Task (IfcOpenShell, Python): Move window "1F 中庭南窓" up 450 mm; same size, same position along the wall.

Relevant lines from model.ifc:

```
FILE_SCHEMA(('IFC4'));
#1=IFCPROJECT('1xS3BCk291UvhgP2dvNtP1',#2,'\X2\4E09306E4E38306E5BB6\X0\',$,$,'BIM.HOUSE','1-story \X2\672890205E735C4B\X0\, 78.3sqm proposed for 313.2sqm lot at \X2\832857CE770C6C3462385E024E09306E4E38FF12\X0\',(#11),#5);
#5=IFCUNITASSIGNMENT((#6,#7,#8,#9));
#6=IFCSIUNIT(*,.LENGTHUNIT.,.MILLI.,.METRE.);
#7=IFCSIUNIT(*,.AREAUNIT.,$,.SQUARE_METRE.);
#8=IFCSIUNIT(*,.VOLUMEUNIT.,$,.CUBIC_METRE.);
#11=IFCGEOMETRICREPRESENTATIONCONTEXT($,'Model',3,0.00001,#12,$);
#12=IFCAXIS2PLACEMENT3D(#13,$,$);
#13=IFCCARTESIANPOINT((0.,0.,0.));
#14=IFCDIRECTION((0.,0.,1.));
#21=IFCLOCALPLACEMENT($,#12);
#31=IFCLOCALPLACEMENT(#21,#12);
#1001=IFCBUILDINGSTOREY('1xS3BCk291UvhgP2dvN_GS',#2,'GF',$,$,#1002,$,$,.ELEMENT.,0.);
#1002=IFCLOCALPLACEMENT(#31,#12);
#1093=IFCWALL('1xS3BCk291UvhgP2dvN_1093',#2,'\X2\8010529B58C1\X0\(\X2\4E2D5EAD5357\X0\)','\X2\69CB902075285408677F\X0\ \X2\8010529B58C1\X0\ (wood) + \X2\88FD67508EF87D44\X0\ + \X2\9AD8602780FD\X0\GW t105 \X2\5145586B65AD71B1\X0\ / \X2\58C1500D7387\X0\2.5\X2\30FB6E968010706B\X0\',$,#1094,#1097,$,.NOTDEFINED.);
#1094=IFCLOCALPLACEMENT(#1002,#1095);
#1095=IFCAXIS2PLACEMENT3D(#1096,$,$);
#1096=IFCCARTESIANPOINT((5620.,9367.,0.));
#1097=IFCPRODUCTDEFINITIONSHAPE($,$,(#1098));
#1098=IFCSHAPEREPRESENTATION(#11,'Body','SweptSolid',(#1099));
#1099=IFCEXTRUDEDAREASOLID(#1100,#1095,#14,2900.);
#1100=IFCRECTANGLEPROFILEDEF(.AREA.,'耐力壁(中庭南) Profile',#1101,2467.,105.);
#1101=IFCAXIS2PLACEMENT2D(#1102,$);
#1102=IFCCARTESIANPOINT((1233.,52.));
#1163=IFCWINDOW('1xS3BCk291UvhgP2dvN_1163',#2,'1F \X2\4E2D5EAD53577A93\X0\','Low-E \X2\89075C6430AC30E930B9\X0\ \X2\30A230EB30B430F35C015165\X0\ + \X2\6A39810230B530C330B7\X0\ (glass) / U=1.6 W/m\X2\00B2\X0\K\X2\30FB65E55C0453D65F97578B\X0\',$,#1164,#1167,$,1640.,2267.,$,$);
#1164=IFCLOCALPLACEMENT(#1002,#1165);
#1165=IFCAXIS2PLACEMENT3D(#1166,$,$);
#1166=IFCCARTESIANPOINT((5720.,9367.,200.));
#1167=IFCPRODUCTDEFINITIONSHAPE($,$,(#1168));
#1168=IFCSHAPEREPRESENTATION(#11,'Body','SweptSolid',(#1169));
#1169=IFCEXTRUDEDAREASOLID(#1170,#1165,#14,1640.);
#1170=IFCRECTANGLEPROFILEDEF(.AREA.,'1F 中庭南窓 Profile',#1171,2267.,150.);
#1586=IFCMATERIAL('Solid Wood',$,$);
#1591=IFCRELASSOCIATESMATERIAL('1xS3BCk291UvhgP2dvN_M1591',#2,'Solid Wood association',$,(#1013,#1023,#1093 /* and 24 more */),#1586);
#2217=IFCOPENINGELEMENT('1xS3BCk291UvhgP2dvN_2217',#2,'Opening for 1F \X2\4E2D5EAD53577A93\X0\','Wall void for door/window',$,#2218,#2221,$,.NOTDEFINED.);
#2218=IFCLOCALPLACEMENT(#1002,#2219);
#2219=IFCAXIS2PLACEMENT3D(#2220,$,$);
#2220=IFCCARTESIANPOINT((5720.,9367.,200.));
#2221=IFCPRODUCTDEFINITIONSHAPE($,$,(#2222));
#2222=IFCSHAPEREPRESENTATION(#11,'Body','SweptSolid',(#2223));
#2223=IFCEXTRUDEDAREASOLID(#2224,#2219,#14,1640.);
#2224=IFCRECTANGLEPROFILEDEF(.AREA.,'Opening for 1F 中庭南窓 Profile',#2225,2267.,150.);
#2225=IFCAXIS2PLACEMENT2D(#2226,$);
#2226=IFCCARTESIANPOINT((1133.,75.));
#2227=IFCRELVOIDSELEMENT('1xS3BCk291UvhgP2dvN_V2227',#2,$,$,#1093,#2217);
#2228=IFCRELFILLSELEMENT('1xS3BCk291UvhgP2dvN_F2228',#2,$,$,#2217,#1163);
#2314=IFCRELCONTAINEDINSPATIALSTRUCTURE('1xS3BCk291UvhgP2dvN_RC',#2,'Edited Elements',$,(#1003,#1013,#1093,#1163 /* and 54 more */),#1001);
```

```python
import numpy as np
import ifcopenshell
import ifcopenshell.api.geometry
import ifcopenshell.util.placement
import ifcopenshell.util.unit

model = ifcopenshell.open("model.ifc")
unit_scale = ifcopenshell.util.unit.calculate_unit_scale(model)

window = model.by_guid("1xS3BCk291UvhgP2dvN_1163")
opening = window.FillsVoids[0].RelatingOpeningElement
dz = 450.0

shift = np.array([0.0, 0.0, dz])
# The window is not placed relative to its opening, so move both.
for product in (opening, window):
    matrix = ifcopenshell.util.placement.get_local_placement(product.ObjectPlacement)
    matrix[:3, 3] += shift
    ifcopenshell.api.geometry.edit_object_placement(model, product=product, matrix=matrix, is_si=False)

print(f"moved by {dz * unit_scale:+.3f} m")

model.write("model_rev.ifc")
```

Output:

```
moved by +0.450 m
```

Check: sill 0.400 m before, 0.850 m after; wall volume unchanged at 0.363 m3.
